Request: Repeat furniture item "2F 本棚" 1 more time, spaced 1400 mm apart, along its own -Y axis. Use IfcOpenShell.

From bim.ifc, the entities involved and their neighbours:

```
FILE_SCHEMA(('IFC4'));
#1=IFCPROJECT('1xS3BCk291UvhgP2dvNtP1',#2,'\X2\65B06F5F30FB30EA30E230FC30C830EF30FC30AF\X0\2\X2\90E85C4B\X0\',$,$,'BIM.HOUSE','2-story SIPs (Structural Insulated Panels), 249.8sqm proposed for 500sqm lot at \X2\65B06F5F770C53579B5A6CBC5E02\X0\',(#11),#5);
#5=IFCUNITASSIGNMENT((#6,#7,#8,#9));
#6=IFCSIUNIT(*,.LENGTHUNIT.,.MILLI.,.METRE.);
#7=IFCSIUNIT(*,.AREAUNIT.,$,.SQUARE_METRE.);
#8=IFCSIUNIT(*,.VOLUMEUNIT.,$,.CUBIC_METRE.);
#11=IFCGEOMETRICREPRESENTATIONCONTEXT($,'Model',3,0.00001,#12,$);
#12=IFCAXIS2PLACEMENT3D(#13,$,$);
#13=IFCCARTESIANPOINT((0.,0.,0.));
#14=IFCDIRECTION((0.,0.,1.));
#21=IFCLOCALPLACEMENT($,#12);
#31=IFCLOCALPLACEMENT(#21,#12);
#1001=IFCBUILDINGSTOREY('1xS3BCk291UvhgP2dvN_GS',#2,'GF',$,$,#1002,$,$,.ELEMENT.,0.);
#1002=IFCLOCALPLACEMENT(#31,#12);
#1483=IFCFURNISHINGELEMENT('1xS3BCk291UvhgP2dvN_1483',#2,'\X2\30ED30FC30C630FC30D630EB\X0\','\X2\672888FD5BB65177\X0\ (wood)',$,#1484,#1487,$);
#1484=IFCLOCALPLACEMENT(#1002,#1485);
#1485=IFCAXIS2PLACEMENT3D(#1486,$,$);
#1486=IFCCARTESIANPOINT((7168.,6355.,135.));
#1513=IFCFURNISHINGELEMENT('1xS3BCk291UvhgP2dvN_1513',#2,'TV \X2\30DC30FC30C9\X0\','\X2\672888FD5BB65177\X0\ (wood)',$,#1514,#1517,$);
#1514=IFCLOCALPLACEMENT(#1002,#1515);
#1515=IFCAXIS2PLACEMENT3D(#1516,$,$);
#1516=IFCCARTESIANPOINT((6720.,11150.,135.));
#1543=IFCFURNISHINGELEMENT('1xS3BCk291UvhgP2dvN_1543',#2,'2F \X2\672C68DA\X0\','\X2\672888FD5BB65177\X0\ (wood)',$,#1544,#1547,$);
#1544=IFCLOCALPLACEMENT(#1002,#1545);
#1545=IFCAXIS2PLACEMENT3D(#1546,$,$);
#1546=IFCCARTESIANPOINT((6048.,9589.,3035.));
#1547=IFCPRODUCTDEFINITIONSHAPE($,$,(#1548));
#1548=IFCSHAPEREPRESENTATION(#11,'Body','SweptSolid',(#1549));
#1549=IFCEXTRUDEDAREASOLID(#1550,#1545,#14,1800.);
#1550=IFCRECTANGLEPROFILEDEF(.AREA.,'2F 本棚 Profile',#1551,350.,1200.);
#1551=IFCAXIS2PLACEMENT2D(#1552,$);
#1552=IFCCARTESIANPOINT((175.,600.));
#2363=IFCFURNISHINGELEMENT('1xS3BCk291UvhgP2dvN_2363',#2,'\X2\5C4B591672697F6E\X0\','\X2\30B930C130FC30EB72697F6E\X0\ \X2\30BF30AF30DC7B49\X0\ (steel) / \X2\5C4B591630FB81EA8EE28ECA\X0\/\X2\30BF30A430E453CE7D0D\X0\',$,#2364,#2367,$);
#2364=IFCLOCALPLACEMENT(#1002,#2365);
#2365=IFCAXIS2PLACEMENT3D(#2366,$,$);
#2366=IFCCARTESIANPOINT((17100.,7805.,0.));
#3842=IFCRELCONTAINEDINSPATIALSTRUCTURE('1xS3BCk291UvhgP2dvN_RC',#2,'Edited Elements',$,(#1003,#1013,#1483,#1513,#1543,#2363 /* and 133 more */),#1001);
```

```python
import ifcopenshell
import ifcopenshell.api.geometry
import ifcopenshell.api.root
import ifcopenshell.util.element
import ifcopenshell.util.placement
import ifcopenshell.util.unit

model = ifcopenshell.open("bim.ifc")
unit_scale = ifcopenshell.util.unit.calculate_unit_scale(model)


def reuse_history(source, copy):
    """copy_class also copies each property set's owner history, people and application; keep the originals."""
    for rel in copy.IsDefinedBy:
        if rel.is_a("IfcRelDefinesByProperties") and (history := rel.RelatingPropertyDefinition.OwnerHistory):
            rel.RelatingPropertyDefinition.OwnerHistory = source.OwnerHistory
            ifcopenshell.util.element.remove_deep2(model, history)


source = model.by_guid("1xS3BCk291UvhgP2dvN_1543")
base = ifcopenshell.util.placement.get_local_placement(source.ObjectPlacement)
step = -base[:3, 1] * 1.4 / unit_scale

for i in range(1, 2):
    copy = ifcopenshell.api.root.copy_class(model, product=source)
    copy.Representation = ifcopenshell.util.element.copy_deep(
        model, source.Representation, exclude=["IfcGeometricRepresentationContext", "IfcRepresentationMap"]
    )
    reuse_history(source, copy)
    matrix = base.copy()
    matrix[:3, 3] += i * step
    print("added at", matrix[:3, 3].round(3) + 0.0)
    ifcopenshell.api.geometry.edit_object_placement(model, product=copy, matrix=matrix, is_si=False)

model.write("bim_rev.ifc")
```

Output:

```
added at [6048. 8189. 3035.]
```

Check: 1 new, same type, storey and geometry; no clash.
